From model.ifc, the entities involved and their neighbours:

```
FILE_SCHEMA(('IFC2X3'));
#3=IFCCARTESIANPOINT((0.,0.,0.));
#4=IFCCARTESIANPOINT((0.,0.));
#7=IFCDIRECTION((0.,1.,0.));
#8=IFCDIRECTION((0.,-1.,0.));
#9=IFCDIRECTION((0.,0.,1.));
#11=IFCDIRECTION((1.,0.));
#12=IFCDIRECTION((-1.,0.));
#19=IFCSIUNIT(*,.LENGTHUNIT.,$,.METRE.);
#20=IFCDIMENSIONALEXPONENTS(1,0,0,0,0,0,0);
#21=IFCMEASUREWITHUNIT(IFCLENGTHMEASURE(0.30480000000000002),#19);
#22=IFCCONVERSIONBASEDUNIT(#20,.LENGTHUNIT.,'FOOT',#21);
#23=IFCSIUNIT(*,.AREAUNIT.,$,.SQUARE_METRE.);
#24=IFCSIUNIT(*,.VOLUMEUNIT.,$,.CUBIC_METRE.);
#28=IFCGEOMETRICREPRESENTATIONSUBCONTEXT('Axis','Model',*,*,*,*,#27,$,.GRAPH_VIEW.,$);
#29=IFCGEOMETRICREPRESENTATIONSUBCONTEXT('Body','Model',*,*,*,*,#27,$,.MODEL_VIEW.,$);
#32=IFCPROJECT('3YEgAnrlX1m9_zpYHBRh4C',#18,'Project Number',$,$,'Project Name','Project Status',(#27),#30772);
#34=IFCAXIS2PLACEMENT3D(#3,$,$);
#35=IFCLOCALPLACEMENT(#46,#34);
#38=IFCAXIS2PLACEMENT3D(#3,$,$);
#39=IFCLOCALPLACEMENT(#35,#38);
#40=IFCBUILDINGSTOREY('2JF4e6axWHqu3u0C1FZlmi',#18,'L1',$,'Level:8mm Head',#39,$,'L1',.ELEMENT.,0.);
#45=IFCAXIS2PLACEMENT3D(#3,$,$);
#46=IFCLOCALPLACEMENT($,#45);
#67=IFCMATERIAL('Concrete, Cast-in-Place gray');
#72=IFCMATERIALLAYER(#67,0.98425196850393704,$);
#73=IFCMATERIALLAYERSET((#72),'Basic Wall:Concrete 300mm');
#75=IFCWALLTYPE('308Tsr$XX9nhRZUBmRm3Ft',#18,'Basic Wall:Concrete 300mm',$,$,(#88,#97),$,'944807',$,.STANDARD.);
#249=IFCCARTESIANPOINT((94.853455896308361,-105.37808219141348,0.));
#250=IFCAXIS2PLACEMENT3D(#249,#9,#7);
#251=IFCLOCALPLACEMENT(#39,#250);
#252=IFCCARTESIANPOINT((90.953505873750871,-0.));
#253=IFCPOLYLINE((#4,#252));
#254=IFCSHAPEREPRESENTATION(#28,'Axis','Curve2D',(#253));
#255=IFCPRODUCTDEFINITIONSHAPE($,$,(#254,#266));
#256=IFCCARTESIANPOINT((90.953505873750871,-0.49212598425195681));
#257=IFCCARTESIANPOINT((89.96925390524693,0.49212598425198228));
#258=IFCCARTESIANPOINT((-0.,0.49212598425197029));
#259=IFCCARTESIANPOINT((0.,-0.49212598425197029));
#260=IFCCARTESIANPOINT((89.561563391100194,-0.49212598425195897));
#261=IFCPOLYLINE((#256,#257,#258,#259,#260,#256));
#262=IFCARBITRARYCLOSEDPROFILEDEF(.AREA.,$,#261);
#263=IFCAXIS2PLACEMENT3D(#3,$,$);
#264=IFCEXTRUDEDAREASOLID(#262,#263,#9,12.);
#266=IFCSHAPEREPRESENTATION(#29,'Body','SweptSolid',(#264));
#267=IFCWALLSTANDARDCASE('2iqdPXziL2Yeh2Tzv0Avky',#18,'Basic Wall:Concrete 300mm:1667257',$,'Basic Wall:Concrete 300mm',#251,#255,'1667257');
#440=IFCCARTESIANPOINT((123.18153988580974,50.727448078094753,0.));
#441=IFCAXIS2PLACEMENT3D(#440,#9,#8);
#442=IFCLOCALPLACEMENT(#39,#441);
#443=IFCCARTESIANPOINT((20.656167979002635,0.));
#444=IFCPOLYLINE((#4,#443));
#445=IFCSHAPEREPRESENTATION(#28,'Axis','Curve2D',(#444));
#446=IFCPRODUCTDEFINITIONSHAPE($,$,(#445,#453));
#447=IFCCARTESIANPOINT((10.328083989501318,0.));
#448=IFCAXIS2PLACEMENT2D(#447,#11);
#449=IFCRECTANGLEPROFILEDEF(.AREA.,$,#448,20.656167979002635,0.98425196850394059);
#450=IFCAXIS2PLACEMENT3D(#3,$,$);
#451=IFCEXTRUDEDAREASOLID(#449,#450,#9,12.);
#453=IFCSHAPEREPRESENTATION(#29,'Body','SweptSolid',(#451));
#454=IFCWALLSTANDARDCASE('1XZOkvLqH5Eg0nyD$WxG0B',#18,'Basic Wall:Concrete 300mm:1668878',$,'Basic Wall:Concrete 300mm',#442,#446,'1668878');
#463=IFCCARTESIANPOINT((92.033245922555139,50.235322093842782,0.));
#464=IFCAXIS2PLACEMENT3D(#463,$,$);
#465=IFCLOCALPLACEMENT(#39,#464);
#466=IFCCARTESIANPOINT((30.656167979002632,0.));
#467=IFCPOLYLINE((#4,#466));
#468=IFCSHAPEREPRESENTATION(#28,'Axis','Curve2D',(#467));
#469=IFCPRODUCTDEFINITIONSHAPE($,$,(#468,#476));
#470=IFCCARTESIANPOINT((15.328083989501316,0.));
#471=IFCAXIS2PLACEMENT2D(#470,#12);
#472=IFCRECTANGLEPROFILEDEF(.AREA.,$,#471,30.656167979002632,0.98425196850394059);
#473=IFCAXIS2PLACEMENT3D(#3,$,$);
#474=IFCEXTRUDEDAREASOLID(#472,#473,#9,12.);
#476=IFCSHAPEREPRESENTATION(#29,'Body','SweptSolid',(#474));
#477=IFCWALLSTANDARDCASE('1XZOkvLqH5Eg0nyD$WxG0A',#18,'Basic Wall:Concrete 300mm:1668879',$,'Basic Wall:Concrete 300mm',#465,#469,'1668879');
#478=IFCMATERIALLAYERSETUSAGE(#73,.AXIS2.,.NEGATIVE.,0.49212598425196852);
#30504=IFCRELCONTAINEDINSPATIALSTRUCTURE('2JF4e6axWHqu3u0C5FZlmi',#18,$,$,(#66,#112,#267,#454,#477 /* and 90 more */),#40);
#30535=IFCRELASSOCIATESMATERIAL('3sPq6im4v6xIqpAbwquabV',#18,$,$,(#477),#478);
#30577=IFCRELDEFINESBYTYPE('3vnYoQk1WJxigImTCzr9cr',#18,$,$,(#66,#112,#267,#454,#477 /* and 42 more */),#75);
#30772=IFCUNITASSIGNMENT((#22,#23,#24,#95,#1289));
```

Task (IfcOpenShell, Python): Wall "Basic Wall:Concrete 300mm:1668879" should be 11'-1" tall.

```python
import ifcopenshell
import ifcopenshell.geom
import ifcopenshell.util.representation
import ifcopenshell.util.shape
import ifcopenshell.util.unit

model = ifcopenshell.open("model.ifc")
unit_scale = ifcopenshell.util.unit.calculate_unit_scale(model)
settings = ifcopenshell.geom.settings()


def volume(element):
    """Net volume in cubic metres, openings subtracted."""
    shape = ifcopenshell.geom.create_shape(settings, element)
    return ifcopenshell.util.shape.get_volume(shape.geometry)


wall = model.by_guid("1XZOkvLqH5Eg0nyD$WxG0A")
before = volume(wall)

body = ifcopenshell.util.representation.get_representation(wall, "Model", "Body")
solid = body.Items[0]
old_height = solid.Depth
solid.Depth = 133 * 0.0254 / unit_scale
after = volume(wall)

print(f"height {old_height:g} -> {solid.Depth:g}, volume {before:.3f} -> {after:.3f} m3")

model.write("model_updated.ifc")
```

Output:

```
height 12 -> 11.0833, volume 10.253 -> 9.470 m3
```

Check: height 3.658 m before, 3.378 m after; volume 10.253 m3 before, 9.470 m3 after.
